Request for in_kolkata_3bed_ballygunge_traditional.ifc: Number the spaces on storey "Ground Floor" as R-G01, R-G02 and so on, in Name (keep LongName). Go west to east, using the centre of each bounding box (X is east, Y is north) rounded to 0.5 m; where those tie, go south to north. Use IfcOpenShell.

First a look at what the model holds.

```python
import ifcopenshell
import ifcopenshell.util.element
import ifcopenshell.util.placement

model = ifcopenshell.open("in_kolkata_3bed_ballygunge_traditional.ifc")
print(model.schema)
storey = next(s for s in model.by_type("IfcBuildingStorey") if s.Name == "Ground Floor")
spaces = [e for e in ifcopenshell.util.element.get_decomposition(storey) if e.is_a("IfcSpace")]
for e in sorted(spaces, key=lambda e: e.id()):
    origin = ifcopenshell.util.placement.get_local_placement(e.ObjectPlacement)[:3, 3]
    print(e.id(), e.Name, e.LongName, origin.round(2) + 0.0, sep=" | ")
```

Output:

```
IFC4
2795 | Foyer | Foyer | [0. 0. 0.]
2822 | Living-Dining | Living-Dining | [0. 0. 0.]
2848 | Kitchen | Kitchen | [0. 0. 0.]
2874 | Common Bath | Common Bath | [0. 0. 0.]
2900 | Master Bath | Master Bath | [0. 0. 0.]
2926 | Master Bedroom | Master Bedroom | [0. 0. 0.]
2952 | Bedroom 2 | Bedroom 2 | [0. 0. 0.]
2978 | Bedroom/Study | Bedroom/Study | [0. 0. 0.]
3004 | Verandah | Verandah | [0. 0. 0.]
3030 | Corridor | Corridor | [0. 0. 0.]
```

```python
import ifcopenshell
import ifcopenshell.geom
import ifcopenshell.util.element
import ifcopenshell.util.shape

model = ifcopenshell.open("in_kolkata_3bed_ballygunge_traditional.ifc")
settings = ifcopenshell.geom.settings()
settings.set("use-world-coords", True)


def centre(element):
    shape = ifcopenshell.geom.create_shape(settings, element)
    return ifcopenshell.util.shape.get_bbox_centroid(shape.geometry)


storey = next(s for s in model.by_type("IfcBuildingStorey") if s.Name == "Ground Floor")
spaces = [e for e in ifcopenshell.util.element.get_decomposition(storey) if e.is_a("IfcSpace")]

# Insertion points can sit at a corner or the storey origin, so sort by the geometry (in metres).
centres = {e: centre(e) for e in spaces}
spaces.sort(key=lambda e: (round(centres[e][0] / 0.5), centres[e][1]))

for i, e in enumerate(spaces, start=1):
    number = f"R-G{i:02d}"
    e.Name = number
    print(e.id(), number)

model.write("in_kolkata_3bed_ballygunge_traditional_edited.ifc")
```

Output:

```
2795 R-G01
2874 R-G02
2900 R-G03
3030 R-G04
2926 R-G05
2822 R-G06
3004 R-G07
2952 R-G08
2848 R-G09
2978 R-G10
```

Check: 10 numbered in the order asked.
